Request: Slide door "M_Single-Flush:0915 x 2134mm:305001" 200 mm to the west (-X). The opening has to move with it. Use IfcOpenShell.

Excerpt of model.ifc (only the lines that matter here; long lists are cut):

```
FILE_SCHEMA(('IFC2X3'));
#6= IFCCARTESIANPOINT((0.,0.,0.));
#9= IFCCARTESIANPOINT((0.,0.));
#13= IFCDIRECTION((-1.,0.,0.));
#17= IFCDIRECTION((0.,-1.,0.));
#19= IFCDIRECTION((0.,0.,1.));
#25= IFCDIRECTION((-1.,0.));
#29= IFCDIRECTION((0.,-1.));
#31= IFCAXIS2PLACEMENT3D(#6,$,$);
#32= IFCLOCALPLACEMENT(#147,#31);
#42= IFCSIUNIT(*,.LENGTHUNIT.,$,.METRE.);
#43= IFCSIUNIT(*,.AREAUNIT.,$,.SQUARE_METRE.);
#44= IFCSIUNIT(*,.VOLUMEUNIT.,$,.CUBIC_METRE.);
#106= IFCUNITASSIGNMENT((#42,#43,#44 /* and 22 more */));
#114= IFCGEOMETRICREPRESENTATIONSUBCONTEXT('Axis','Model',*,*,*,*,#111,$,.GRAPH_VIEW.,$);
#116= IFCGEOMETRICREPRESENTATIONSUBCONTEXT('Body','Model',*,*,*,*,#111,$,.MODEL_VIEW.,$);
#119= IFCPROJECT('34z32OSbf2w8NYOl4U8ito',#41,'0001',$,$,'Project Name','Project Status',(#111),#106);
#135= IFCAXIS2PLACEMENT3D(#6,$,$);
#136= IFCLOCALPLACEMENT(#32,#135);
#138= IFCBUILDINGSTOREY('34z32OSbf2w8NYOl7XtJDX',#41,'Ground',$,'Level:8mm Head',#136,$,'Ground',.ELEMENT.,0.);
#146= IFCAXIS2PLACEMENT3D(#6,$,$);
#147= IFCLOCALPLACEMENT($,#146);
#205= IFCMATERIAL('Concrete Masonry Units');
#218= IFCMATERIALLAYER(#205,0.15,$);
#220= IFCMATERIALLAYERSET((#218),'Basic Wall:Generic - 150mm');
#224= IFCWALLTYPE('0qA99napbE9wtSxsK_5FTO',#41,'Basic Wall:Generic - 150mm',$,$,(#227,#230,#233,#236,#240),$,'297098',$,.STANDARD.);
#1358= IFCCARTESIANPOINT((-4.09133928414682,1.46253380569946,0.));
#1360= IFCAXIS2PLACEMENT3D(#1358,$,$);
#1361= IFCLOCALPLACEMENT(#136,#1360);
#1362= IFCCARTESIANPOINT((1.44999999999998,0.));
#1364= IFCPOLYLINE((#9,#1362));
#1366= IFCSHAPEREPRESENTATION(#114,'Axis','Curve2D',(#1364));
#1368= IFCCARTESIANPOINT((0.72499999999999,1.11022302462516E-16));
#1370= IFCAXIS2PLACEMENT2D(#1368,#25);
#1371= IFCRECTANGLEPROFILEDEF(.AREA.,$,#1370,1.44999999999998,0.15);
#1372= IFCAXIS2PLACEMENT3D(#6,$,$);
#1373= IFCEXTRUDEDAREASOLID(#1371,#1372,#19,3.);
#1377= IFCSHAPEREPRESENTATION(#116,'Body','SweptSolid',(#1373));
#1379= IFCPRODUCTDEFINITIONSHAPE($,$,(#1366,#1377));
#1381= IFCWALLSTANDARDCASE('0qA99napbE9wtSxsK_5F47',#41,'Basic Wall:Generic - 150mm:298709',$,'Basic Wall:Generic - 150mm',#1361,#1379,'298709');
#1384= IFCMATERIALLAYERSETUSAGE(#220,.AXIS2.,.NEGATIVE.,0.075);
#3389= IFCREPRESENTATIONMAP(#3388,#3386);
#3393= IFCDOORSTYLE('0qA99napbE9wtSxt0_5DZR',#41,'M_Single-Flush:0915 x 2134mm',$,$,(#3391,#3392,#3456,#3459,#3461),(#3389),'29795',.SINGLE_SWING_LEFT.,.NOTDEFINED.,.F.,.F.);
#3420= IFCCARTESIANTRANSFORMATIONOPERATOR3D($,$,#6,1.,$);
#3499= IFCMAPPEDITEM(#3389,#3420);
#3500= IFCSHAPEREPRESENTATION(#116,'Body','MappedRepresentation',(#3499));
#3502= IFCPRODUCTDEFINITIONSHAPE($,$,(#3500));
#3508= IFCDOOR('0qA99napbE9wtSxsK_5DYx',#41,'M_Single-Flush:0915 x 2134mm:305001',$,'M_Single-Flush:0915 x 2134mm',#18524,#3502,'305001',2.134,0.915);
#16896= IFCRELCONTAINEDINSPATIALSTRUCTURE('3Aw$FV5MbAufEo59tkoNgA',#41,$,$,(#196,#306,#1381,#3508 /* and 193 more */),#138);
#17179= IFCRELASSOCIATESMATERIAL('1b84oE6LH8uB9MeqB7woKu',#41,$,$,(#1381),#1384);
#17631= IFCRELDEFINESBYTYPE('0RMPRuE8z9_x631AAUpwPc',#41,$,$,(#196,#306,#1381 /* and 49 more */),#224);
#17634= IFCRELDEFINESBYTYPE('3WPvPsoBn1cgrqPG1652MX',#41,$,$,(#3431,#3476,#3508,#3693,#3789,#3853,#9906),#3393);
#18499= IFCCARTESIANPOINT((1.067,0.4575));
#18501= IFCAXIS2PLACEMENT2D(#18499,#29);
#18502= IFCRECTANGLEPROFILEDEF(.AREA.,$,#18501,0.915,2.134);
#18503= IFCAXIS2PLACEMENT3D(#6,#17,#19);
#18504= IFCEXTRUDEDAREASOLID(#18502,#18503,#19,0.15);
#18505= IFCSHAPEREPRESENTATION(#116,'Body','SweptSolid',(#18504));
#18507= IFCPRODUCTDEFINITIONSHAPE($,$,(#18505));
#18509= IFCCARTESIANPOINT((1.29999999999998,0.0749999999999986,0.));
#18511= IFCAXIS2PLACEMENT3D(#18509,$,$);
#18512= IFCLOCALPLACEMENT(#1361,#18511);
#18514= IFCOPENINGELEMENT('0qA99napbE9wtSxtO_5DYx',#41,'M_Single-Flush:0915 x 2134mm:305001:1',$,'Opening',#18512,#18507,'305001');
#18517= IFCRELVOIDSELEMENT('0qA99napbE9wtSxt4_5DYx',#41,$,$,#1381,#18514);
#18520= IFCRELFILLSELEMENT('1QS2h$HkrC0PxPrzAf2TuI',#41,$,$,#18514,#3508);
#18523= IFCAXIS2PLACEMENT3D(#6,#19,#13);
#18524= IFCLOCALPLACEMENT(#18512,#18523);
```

```python
import ifcopenshell
import ifcopenshell.api.geometry
import ifcopenshell.util.placement
import ifcopenshell.util.unit

model = ifcopenshell.open("model.ifc")
unit_scale = ifcopenshell.util.unit.calculate_unit_scale(model)

door = model.by_guid("0qA99napbE9wtSxsK_5DYx")
opening = door.FillsVoids[0].RelatingOpeningElement
wall = opening.VoidsElements[0].RelatingBuildingElement

wall_matrix = ifcopenshell.util.placement.get_local_placement(wall.ObjectPlacement)
shift = wall_matrix[:3, 0] * -0.2 / unit_scale
before = ifcopenshell.util.placement.get_local_placement(door.ObjectPlacement)[:3, 3].copy()

# The door is placed relative to its opening, so it follows when the opening moves.
matrix = ifcopenshell.util.placement.get_local_placement(opening.ObjectPlacement)
matrix[:3, 3] += shift
ifcopenshell.api.geometry.edit_object_placement(
    model, product=opening, matrix=matrix, is_si=False, should_transform_children=True
)

after = ifcopenshell.util.placement.get_local_placement(door.ObjectPlacement)[:3, 3]
print("door moved by", (after - before).round(3) + 0.0)

model.write("model_rev.ifc")
```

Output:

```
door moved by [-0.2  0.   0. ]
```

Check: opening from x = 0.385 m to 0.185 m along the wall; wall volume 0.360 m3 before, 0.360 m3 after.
